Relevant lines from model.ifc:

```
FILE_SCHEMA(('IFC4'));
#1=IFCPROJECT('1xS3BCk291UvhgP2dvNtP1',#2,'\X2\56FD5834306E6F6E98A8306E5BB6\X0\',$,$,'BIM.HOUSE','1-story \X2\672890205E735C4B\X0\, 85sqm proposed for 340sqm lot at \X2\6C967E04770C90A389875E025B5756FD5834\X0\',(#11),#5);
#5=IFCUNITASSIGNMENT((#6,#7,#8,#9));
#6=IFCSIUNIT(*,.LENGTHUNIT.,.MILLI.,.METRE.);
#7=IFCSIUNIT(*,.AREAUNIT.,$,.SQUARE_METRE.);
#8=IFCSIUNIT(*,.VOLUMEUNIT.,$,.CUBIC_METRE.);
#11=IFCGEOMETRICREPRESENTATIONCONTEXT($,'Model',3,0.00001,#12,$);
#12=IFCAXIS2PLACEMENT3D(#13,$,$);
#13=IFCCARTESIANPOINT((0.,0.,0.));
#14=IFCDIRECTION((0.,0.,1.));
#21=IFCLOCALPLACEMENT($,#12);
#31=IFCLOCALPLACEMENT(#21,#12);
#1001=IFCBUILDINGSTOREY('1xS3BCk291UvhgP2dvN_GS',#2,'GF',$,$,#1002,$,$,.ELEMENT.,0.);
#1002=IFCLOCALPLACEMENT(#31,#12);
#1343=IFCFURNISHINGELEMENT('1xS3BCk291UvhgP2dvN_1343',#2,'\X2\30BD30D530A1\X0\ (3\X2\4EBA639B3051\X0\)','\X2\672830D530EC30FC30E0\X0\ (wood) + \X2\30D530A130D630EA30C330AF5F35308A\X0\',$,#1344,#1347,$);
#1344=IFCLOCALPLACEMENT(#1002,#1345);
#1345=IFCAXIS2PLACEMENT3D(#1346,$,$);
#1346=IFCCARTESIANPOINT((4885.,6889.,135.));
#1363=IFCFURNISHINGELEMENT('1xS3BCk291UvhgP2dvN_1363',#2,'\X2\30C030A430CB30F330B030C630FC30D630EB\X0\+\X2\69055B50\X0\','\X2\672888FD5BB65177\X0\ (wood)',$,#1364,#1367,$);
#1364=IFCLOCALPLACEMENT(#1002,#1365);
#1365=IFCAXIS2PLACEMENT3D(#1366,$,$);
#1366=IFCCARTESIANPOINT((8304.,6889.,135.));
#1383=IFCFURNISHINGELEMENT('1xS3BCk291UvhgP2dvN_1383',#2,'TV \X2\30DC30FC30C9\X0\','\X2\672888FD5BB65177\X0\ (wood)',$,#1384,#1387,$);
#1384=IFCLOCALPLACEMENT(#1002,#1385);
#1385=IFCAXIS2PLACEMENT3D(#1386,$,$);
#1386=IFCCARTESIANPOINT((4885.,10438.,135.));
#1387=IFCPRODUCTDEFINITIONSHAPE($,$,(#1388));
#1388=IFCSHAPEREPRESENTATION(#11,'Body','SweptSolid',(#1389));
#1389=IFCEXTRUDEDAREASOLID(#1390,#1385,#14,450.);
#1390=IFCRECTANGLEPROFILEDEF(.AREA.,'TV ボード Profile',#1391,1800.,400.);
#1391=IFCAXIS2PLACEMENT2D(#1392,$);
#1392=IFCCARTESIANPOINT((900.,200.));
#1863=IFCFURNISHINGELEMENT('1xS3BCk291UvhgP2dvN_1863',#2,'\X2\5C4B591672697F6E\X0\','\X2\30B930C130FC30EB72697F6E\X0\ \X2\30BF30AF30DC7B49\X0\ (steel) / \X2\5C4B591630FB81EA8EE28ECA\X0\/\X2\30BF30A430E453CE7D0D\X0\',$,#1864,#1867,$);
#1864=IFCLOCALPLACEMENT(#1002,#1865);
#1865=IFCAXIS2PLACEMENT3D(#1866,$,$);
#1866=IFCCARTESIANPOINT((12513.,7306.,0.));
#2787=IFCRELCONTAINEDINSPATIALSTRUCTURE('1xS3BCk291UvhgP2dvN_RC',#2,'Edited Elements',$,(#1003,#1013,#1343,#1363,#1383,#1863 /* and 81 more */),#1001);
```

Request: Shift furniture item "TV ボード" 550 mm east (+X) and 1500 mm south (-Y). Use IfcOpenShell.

```python
import ifcopenshell
import ifcopenshell.api.geometry
import ifcopenshell.util.placement

model = ifcopenshell.open("model.ifc")

item = model.by_guid("1xS3BCk291UvhgP2dvN_1383")
matrix = ifcopenshell.util.placement.get_local_placement(item.ObjectPlacement)
matrix[0, 3] += 550.0
matrix[1, 3] -= 1500.0
ifcopenshell.api.geometry.edit_object_placement(model, product=item, matrix=matrix, is_si=False)

print(ifcopenshell.util.placement.get_local_placement(item.ObjectPlacement).round(3) + 0.0)

model.write("model-out.ifc")
```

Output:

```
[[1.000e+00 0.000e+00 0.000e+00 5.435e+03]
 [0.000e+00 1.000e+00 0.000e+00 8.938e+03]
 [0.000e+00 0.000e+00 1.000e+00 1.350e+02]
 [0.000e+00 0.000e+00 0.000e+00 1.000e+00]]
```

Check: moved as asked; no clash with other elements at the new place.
